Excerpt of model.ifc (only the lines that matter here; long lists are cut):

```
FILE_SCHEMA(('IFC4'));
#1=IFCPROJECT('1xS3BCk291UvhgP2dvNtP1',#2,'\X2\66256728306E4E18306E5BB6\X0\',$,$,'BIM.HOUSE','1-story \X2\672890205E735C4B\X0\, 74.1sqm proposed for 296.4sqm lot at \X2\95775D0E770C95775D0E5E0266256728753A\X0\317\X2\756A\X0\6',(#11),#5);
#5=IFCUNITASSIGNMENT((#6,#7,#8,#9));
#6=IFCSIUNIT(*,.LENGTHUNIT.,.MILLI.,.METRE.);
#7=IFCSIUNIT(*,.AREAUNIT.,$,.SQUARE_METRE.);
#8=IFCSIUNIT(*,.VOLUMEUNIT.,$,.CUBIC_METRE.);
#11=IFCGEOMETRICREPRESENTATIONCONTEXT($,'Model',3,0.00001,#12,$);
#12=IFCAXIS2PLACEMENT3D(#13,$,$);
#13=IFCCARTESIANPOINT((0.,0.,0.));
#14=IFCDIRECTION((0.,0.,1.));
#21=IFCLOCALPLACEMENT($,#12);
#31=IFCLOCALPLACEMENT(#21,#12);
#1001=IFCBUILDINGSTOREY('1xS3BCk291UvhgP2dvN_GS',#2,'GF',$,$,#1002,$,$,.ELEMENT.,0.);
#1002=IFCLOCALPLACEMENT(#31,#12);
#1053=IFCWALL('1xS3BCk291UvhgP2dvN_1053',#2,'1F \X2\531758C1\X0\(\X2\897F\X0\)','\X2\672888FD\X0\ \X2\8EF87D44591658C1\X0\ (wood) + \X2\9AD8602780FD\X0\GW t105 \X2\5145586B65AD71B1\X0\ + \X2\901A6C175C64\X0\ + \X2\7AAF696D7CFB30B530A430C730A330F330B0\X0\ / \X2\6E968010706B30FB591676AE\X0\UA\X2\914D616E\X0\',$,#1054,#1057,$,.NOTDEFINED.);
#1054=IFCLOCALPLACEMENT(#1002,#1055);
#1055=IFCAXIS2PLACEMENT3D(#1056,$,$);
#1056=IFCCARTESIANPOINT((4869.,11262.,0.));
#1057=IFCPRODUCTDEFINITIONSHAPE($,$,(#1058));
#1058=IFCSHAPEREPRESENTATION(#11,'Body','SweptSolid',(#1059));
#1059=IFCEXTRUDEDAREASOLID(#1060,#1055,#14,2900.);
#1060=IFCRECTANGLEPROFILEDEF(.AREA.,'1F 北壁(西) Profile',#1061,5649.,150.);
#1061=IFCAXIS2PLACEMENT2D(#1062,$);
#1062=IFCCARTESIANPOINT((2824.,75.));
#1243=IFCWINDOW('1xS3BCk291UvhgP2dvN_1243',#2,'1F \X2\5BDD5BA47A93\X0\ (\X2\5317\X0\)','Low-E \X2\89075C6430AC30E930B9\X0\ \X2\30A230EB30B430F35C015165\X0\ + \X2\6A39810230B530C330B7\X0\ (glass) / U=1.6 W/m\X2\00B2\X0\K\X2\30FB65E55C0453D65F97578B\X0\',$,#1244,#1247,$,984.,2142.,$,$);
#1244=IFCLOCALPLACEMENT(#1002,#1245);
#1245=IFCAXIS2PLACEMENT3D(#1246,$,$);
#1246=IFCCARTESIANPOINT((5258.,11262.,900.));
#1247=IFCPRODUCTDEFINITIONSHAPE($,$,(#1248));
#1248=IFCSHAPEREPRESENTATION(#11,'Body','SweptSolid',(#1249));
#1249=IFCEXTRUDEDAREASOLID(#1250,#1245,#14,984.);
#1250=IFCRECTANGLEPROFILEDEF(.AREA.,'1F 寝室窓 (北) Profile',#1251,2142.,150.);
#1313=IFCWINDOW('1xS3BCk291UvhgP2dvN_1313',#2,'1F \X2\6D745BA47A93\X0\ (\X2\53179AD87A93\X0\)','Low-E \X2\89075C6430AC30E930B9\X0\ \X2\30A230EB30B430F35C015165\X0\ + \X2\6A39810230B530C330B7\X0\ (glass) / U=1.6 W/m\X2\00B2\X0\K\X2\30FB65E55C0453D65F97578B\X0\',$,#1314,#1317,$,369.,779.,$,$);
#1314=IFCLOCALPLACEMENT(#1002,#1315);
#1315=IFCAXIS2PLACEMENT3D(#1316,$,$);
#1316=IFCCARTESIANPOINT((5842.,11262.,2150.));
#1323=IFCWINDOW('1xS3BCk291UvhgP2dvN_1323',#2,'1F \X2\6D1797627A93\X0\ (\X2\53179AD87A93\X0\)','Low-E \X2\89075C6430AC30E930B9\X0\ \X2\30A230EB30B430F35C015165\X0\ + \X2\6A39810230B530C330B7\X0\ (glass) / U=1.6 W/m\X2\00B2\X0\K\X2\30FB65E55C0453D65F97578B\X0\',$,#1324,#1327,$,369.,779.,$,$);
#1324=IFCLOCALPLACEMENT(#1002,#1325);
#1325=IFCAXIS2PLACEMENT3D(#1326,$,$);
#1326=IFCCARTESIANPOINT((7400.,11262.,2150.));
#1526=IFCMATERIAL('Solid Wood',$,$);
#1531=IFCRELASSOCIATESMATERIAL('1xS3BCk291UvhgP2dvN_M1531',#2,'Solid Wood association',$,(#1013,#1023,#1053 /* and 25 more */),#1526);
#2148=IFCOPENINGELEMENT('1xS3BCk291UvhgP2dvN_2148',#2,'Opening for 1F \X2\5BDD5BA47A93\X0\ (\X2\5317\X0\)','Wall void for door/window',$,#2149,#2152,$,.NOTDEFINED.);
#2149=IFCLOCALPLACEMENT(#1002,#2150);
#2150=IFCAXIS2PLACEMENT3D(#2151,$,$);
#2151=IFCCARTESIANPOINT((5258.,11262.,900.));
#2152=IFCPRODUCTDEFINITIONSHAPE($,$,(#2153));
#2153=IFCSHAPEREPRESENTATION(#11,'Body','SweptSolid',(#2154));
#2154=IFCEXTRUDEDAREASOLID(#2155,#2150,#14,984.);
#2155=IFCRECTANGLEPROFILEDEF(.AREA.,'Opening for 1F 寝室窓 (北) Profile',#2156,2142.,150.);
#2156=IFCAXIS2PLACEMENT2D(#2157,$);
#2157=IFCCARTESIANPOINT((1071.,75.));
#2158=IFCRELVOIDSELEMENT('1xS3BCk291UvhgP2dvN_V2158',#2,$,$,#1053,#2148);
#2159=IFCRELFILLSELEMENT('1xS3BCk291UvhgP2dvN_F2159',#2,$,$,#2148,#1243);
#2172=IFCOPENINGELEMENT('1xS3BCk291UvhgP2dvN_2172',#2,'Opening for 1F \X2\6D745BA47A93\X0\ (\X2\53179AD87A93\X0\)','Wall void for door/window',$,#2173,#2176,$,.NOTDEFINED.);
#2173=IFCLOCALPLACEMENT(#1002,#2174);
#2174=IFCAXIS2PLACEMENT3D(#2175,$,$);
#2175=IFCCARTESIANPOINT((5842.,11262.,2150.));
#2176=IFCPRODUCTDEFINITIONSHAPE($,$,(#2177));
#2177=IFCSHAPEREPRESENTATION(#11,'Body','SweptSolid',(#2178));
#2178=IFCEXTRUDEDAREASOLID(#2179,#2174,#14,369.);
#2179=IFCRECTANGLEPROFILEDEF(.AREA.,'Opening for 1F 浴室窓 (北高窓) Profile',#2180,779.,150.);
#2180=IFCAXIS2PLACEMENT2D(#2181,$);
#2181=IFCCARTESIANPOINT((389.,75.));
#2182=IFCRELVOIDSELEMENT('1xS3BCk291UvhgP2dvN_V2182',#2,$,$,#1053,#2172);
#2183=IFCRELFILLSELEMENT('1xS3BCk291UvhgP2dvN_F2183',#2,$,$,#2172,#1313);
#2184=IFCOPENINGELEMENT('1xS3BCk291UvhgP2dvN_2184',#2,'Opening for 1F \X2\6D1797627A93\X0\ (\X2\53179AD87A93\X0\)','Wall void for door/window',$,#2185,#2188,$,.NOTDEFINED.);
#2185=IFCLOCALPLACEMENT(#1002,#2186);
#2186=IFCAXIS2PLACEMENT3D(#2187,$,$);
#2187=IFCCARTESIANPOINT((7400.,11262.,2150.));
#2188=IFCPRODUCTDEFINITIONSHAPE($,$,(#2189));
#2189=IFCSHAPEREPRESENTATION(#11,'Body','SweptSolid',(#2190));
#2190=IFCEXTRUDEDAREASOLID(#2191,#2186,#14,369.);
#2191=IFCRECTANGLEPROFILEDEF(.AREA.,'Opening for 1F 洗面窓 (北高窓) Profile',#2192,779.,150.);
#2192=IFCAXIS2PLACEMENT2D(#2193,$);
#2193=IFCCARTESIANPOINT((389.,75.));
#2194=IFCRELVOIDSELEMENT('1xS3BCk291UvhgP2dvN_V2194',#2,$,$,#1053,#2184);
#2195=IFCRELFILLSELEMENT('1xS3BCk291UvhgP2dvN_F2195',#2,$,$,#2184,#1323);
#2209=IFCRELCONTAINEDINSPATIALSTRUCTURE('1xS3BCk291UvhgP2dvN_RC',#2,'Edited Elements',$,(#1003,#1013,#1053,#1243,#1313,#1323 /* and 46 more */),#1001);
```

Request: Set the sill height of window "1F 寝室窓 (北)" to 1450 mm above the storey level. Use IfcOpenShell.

```python
import numpy as np
import ifcopenshell
import ifcopenshell.api.geometry
import ifcopenshell.geom
import ifcopenshell.util.element
import ifcopenshell.util.placement
import ifcopenshell.util.shape
import ifcopenshell.util.unit

model = ifcopenshell.open("model.ifc")
unit_scale = ifcopenshell.util.unit.calculate_unit_scale(model)

window = model.by_id(1243)
opening = window.FillsVoids[0].RelatingOpeningElement
storey = ifcopenshell.util.element.get_container(window, ifc_class="IfcBuildingStorey")
level = ifcopenshell.util.placement.get_local_placement(storey.ObjectPlacement)[2, 3]

# The opening's origin need not be at the sill, so measure its lowest point.
shape = ifcopenshell.geom.create_shape(ifcopenshell.geom.settings(), opening)
bottom = ifcopenshell.util.shape.get_shape_bottom_elevation(shape, shape.geometry) / unit_scale
dz = level + 1.45 / unit_scale - bottom

shift = np.array([0.0, 0.0, dz])
# The window is not placed relative to its opening, so move both.
for product in (opening, window):
    matrix = ifcopenshell.util.placement.get_local_placement(product.ObjectPlacement)
    matrix[:3, 3] += shift
    ifcopenshell.api.geometry.edit_object_placement(model, product=product, matrix=matrix, is_si=False)

print(f"moved by {dz * unit_scale:+.3f} m")

model.write("model_updated.ifc")
```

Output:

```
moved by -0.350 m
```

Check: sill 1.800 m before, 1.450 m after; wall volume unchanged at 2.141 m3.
